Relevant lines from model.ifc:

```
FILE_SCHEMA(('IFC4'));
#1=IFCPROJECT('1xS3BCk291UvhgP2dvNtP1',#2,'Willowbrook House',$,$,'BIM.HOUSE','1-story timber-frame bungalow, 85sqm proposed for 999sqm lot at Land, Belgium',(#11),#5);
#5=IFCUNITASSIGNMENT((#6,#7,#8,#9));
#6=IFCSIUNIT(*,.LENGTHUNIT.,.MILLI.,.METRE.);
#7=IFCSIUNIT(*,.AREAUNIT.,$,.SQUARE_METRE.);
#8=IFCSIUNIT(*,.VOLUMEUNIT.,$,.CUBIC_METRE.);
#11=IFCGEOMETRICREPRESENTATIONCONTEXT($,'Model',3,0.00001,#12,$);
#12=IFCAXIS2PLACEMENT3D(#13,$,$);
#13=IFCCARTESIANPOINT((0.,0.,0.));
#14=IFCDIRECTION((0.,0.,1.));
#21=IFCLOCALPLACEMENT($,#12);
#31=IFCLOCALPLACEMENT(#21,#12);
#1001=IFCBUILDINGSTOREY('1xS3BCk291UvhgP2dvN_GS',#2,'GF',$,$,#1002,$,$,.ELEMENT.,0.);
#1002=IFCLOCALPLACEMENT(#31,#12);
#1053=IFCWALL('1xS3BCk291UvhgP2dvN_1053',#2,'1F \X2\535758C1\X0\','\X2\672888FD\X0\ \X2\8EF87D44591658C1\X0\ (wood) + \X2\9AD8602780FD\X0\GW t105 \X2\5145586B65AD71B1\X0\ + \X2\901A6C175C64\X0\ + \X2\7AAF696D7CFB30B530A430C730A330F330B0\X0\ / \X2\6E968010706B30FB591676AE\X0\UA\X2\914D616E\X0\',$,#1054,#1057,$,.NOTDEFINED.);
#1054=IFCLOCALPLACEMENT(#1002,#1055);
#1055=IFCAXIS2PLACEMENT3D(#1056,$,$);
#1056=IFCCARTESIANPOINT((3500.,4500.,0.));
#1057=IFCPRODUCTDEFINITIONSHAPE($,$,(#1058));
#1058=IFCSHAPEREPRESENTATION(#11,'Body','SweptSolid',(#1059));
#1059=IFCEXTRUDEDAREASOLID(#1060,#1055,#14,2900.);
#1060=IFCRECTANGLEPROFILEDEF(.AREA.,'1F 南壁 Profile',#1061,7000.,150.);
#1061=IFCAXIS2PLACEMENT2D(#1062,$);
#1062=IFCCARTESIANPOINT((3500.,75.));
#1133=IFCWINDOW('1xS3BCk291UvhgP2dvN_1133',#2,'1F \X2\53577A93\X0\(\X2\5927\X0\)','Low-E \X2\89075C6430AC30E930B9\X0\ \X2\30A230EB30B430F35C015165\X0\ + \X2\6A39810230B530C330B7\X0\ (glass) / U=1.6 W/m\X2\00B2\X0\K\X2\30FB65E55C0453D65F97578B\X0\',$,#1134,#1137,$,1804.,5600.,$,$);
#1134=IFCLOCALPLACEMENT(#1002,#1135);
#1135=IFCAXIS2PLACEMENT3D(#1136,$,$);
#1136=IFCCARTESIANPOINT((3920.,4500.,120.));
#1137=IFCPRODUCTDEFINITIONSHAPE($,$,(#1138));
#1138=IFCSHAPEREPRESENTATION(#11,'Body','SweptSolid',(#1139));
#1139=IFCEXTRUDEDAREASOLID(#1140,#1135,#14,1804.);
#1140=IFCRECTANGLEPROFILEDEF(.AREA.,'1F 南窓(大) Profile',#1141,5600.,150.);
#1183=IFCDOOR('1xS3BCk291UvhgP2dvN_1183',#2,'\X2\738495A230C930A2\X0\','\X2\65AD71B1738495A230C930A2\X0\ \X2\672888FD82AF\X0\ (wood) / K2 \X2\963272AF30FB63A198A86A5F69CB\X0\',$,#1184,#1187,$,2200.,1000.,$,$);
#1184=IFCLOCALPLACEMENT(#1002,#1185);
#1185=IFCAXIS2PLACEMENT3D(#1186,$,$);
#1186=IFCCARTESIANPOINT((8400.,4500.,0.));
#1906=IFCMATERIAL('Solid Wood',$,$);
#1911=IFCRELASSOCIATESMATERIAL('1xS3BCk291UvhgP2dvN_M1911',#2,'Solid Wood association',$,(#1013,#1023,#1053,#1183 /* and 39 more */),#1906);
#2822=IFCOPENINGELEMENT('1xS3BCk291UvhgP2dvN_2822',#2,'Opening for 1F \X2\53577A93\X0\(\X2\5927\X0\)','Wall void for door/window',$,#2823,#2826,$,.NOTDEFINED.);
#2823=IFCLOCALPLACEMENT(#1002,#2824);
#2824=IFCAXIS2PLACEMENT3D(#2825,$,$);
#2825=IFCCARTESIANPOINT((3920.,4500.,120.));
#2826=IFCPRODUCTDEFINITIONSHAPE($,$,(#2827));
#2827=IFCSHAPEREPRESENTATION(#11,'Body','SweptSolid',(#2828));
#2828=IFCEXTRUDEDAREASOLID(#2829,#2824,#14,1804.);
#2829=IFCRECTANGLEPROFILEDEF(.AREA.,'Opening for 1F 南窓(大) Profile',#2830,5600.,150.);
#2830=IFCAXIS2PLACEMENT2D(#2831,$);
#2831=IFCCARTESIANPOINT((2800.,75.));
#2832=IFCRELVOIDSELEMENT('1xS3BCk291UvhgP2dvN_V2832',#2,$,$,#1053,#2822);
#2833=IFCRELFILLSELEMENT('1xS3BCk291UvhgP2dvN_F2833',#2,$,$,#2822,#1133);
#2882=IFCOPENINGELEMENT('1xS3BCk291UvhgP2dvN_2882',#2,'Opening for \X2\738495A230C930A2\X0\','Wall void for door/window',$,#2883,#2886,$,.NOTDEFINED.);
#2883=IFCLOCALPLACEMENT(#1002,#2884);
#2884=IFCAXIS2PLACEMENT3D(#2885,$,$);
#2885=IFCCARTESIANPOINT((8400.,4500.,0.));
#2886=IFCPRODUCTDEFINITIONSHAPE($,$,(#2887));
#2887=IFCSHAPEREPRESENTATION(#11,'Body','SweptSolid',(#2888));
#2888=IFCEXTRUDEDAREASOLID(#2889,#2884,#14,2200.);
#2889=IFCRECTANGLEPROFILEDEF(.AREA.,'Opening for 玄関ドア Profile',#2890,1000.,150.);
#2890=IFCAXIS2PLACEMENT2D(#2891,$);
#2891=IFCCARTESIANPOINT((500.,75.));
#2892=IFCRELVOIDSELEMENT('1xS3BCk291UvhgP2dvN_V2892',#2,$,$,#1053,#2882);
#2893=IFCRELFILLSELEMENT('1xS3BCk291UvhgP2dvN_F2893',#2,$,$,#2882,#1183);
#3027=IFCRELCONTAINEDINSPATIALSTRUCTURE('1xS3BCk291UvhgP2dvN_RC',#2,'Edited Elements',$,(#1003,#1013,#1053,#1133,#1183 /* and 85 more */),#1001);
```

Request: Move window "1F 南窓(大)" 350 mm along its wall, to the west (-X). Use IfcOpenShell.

```python
import ifcopenshell
import ifcopenshell.api.geometry
import ifcopenshell.util.placement
import ifcopenshell.util.unit

model = ifcopenshell.open("model.ifc")
unit_scale = ifcopenshell.util.unit.calculate_unit_scale(model)

window = model.by_guid("1xS3BCk291UvhgP2dvN_1133")
opening = window.FillsVoids[0].RelatingOpeningElement
wall = opening.VoidsElements[0].RelatingBuildingElement

wall_matrix = ifcopenshell.util.placement.get_local_placement(wall.ObjectPlacement)
shift = wall_matrix[:3, 0] * -0.35 / unit_scale
before = ifcopenshell.util.placement.get_local_placement(window.ObjectPlacement)[:3, 3].copy()

# The window is not placed relative to its opening, so move both.
for product in (opening, window):
    matrix = ifcopenshell.util.placement.get_local_placement(product.ObjectPlacement)
    matrix[:3, 3] += shift
    ifcopenshell.api.geometry.edit_object_placement(model, product=product, matrix=matrix, is_si=False)

after = ifcopenshell.util.placement.get_local_placement(window.ObjectPlacement)[:3, 3]
print("window moved by", (after - before).round(3) + 0.0)

model.write("model-out.ifc")
```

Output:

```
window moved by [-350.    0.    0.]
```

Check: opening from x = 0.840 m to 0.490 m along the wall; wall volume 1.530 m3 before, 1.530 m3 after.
